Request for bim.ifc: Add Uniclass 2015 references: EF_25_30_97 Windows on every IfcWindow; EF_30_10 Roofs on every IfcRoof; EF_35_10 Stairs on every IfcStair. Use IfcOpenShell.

First a look at what the model holds.

```python
import ifcopenshell

model = ifcopenshell.open("bim.ifc")
print(model.schema)
print("classifications:", [c.Name for c in model.by_type("IfcClassification")])
for ifc_class in ("IfcDoor", "IfcRoof", "IfcStair", "IfcWall", "IfcWindow"):
    print(ifc_class, len(model.by_type(ifc_class)))
```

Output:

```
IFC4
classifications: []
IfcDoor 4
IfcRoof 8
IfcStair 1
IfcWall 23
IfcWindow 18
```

```python
import ifcopenshell
import ifcopenshell.api.classification

model = ifcopenshell.open("bim.ifc")

system = ifcopenshell.api.classification.add_classification(model, classification="Uniclass 2015")

codes = {
    "IfcWindow": ("EF_25_30_97", "Windows"),
    "IfcRoof": ("EF_30_10", "Roofs"),
    "IfcStair": ("EF_35_10", "Stairs"),
}
for ifc_class, (code, name) in codes.items():
    products = model.by_type(ifc_class)
    ifcopenshell.api.classification.add_reference(
        model, products=products, classification=system, identification=code, name=name
    )
    print(code, len(products))

model.write("bim_rev.ifc")
```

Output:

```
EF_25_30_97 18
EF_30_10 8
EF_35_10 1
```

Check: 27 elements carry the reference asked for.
